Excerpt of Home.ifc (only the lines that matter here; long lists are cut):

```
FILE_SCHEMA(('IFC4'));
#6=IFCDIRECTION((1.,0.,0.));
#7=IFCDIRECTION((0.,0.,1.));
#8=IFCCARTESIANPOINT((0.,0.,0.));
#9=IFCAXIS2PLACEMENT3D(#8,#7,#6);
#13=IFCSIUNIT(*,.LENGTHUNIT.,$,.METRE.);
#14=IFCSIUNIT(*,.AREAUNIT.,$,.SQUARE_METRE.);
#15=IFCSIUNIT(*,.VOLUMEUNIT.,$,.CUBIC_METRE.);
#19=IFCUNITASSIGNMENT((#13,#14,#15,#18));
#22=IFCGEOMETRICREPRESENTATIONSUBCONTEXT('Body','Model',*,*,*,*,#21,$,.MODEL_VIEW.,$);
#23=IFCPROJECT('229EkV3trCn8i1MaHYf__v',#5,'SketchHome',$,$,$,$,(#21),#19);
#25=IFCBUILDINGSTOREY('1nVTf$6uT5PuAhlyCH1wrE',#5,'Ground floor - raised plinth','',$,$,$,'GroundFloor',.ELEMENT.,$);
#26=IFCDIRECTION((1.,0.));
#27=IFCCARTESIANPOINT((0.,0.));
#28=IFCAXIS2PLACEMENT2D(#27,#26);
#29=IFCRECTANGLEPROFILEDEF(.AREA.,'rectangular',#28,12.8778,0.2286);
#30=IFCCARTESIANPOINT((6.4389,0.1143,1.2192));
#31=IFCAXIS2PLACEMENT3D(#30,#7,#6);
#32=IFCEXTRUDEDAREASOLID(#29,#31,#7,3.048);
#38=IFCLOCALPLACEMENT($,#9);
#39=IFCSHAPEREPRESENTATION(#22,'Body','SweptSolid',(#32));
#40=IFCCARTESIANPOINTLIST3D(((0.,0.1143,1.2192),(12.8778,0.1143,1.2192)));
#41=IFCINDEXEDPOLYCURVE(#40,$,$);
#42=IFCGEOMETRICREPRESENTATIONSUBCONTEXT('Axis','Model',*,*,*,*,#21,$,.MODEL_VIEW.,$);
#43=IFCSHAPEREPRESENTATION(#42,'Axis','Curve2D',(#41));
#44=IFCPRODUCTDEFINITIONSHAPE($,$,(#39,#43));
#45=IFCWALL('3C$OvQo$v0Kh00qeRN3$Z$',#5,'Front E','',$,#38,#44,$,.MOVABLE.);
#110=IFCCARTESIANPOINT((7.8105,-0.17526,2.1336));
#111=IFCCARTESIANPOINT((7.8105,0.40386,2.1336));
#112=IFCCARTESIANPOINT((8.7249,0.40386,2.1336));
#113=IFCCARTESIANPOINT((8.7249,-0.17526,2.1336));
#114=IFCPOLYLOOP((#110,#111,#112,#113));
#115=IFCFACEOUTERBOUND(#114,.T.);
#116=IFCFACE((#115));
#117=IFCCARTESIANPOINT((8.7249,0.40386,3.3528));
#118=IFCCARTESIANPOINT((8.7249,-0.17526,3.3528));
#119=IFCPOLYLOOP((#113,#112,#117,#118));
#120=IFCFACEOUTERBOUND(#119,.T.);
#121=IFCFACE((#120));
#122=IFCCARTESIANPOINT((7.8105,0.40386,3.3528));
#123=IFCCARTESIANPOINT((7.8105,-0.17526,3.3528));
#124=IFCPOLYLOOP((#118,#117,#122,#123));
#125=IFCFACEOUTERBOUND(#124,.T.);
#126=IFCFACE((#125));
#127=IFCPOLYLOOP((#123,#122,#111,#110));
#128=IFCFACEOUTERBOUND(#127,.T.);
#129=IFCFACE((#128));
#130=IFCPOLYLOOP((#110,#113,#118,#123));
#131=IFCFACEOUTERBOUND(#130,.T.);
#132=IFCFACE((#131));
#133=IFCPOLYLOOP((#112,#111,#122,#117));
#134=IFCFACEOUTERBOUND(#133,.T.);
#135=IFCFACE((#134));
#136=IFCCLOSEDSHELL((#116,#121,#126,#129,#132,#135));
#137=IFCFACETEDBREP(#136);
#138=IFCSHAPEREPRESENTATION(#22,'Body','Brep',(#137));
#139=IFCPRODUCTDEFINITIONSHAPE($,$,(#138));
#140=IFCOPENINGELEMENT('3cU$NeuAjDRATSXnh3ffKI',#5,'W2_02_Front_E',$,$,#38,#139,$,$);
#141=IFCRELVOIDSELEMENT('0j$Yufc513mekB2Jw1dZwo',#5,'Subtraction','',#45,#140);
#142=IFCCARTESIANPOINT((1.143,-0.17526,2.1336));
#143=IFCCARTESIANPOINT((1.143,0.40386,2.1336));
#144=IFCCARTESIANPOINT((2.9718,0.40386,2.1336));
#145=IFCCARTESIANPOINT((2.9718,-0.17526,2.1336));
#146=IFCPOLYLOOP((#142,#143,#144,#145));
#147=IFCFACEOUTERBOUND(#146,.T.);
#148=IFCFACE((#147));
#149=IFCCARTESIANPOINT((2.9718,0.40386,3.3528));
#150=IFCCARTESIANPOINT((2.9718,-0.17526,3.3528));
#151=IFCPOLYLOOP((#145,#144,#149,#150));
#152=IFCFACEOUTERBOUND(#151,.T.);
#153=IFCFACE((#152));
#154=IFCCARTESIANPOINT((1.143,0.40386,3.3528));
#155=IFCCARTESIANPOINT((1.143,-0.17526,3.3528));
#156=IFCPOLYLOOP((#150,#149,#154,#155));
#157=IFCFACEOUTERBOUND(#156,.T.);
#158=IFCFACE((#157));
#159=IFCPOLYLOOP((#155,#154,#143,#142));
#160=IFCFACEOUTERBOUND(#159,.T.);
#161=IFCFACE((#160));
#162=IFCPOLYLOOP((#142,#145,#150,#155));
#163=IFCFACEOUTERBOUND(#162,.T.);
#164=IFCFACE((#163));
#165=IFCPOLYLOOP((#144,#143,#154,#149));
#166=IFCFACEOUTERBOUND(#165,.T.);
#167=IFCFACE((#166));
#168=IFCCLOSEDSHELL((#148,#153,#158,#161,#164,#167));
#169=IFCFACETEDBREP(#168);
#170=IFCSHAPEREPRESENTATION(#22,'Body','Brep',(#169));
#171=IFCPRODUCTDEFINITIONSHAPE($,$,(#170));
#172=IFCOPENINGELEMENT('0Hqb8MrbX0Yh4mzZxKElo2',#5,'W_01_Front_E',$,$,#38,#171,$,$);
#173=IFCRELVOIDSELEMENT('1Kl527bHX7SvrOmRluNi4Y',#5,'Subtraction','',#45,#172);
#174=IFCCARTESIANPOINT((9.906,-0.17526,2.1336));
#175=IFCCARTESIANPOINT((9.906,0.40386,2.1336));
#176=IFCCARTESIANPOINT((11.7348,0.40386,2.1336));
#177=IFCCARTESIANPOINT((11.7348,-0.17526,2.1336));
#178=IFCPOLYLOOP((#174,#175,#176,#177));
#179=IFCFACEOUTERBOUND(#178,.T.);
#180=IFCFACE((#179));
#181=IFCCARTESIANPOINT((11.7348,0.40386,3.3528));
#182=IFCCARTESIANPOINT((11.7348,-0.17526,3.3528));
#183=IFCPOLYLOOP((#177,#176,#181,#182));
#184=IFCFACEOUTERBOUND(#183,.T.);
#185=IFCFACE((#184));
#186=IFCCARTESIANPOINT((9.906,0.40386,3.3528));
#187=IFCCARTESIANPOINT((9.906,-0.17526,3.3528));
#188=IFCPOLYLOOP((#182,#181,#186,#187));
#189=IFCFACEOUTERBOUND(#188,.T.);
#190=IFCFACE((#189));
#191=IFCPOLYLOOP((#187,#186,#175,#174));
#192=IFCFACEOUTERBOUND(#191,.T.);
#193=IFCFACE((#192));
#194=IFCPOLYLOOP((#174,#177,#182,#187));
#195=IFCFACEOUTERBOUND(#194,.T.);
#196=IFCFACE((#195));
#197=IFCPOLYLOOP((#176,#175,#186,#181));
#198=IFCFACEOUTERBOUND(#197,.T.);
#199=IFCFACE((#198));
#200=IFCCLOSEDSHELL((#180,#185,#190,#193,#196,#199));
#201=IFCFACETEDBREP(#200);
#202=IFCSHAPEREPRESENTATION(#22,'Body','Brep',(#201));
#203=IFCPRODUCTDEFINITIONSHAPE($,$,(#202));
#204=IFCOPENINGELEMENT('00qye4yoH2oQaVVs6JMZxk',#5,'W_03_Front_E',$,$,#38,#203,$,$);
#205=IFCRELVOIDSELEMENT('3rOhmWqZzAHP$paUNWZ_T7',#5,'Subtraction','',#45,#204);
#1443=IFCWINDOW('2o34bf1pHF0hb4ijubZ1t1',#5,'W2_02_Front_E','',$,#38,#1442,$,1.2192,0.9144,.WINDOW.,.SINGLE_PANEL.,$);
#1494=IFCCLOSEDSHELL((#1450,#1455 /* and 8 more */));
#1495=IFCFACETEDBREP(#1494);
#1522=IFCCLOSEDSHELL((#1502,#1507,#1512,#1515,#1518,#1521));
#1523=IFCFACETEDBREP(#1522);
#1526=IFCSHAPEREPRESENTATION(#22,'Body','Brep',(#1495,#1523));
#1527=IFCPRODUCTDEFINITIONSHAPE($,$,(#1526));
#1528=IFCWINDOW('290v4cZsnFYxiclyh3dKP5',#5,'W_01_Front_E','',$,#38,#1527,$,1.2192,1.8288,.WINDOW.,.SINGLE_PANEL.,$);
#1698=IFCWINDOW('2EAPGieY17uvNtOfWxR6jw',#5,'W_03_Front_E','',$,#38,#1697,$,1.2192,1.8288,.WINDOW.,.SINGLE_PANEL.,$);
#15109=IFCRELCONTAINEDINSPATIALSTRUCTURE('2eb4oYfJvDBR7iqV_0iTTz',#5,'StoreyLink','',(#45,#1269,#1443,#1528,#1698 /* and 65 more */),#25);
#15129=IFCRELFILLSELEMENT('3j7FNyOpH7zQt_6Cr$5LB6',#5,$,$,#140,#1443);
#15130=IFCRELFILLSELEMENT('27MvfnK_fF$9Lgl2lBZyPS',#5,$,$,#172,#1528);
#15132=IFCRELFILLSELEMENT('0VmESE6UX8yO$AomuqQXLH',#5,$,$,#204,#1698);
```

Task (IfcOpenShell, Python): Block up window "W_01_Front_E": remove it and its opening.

```python
import ifcopenshell
import ifcopenshell.api.feature
import ifcopenshell.api.root
import ifcopenshell.geom
import ifcopenshell.util.shape

model = ifcopenshell.open("Home.ifc")
settings = ifcopenshell.geom.settings()


def volume(element):
    """Net volume in cubic metres, openings subtracted."""
    shape = ifcopenshell.geom.create_shape(settings, element)
    return ifcopenshell.util.shape.get_volume(shape.geometry)


window = model.by_guid("290v4cZsnFYxiclyh3dKP5")
opening = window.FillsVoids[0].RelatingOpeningElement
wall = opening.VoidsElements[0].RelatingBuildingElement
before = volume(wall)

ifcopenshell.api.root.remove_product(model, product=window)
ifcopenshell.api.feature.remove_feature(model, feature=opening)

after = volume(wall)

print(f"wall volume {before:.3f} -> {after:.3f} m3")

model.write("Home_rev.ifc")
```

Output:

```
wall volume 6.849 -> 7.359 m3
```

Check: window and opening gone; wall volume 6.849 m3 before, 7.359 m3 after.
